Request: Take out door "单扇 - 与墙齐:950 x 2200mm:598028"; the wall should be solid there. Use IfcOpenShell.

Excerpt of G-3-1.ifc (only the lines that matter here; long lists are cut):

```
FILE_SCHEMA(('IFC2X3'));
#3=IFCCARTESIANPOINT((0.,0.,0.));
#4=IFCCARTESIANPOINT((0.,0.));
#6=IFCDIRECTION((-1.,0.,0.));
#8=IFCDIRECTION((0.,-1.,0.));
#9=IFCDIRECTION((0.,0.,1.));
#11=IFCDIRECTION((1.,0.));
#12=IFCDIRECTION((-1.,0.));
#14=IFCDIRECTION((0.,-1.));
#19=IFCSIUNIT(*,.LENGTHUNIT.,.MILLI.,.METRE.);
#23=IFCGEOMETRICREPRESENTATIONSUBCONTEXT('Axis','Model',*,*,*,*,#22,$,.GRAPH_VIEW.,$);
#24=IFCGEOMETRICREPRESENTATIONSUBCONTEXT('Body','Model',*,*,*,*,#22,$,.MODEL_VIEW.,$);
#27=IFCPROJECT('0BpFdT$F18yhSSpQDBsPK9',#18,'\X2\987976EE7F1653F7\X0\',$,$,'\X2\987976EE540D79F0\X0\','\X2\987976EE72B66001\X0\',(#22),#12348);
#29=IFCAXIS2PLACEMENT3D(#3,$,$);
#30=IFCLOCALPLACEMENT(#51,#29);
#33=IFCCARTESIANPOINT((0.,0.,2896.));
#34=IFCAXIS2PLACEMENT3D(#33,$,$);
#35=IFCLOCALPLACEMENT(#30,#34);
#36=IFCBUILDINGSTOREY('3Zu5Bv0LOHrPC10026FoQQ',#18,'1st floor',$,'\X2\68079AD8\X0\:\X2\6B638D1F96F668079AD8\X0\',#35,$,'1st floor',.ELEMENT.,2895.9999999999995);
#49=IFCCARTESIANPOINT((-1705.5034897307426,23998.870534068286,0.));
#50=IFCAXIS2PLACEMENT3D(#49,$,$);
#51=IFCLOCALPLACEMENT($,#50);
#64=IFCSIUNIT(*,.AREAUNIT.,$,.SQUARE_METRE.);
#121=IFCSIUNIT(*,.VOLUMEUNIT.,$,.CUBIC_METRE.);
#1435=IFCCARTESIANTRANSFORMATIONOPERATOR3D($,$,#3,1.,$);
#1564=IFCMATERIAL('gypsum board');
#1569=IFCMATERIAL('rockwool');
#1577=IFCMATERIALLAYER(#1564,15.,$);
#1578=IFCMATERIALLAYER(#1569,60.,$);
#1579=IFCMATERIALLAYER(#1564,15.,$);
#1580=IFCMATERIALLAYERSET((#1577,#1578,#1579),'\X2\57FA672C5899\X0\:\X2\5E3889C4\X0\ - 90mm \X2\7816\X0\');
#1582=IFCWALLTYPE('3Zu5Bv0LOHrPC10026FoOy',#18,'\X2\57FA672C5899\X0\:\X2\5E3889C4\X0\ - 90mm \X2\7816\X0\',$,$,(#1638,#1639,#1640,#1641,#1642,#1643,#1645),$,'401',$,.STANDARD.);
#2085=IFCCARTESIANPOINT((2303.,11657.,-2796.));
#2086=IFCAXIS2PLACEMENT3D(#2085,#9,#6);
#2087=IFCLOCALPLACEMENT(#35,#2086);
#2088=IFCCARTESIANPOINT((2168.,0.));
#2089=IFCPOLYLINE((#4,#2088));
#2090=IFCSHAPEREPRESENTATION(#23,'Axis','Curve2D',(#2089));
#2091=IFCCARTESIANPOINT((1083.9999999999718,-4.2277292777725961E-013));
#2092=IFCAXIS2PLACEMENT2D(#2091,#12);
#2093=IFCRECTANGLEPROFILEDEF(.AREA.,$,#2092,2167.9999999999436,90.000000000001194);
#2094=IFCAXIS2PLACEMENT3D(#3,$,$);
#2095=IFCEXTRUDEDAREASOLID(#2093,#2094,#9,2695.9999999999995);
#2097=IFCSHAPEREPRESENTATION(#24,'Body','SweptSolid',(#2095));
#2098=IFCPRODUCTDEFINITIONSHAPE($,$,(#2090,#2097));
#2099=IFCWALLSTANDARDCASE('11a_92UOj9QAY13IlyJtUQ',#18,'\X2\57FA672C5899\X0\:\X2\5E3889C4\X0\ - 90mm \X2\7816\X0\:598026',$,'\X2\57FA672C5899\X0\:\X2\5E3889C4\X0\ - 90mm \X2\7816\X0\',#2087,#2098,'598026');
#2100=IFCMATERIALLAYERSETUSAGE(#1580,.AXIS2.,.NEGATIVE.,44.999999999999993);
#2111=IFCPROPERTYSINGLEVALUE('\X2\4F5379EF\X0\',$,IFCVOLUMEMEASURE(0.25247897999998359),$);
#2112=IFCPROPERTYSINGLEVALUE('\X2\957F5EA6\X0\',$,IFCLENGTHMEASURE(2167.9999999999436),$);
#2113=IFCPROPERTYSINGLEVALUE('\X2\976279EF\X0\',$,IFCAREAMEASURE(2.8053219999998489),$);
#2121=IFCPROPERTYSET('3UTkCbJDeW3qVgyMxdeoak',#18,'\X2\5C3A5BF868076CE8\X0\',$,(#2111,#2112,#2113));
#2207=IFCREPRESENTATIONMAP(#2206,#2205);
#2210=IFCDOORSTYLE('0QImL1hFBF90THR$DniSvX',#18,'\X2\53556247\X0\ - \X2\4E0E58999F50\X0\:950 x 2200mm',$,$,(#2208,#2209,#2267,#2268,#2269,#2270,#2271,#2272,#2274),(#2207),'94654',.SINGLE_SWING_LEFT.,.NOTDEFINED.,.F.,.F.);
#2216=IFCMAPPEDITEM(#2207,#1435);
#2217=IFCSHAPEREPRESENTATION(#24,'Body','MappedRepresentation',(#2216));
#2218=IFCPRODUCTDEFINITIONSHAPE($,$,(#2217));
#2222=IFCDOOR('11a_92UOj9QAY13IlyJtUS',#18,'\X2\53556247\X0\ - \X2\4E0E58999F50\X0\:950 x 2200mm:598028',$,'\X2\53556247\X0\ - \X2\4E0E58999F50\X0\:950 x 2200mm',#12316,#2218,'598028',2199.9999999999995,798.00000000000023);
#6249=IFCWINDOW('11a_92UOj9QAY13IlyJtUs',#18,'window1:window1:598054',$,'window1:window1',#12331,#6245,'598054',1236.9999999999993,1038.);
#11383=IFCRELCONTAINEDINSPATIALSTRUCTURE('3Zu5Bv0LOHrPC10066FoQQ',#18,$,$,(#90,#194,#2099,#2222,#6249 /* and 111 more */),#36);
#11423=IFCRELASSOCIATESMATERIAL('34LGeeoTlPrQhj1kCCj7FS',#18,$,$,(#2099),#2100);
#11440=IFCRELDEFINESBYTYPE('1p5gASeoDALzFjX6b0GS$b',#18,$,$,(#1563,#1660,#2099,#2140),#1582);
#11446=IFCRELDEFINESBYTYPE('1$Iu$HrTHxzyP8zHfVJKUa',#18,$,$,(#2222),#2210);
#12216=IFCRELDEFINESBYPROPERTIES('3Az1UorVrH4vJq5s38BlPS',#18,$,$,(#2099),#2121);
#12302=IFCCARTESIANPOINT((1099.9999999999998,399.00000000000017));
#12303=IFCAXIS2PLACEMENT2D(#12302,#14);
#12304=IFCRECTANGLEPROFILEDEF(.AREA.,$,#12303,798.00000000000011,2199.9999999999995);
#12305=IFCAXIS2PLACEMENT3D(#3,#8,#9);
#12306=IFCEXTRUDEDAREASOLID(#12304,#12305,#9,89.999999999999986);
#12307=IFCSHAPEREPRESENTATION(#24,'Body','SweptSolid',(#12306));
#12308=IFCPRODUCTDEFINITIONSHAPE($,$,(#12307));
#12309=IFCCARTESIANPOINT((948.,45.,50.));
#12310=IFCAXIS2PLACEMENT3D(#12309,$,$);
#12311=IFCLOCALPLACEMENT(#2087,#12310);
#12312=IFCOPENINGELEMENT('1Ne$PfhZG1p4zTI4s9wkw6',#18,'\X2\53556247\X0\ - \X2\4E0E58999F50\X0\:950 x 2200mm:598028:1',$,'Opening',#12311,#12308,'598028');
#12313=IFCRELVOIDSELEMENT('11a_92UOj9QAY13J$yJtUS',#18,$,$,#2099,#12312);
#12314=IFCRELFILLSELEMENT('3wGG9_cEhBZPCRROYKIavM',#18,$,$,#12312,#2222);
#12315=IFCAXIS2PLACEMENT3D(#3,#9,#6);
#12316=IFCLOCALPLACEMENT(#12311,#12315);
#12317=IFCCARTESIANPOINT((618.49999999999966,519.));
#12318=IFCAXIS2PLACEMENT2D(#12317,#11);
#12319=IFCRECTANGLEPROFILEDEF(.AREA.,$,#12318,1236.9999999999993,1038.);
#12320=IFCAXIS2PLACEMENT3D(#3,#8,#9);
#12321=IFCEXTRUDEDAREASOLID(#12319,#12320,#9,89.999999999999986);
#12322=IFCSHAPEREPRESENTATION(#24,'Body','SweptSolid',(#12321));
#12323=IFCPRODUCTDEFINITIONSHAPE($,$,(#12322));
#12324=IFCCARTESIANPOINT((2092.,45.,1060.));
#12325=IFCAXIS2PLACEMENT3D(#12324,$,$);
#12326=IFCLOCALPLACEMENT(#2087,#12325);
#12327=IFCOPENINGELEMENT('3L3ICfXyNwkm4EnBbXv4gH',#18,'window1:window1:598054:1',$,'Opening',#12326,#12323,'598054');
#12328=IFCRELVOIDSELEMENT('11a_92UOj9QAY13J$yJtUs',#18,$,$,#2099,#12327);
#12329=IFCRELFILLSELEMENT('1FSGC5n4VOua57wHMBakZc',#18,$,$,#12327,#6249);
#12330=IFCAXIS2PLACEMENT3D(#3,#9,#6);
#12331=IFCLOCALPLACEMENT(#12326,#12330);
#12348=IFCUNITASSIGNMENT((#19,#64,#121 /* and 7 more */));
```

```python
import ifcopenshell
import ifcopenshell.api.feature
import ifcopenshell.api.pset
import ifcopenshell.api.root
import ifcopenshell.geom
import ifcopenshell.util.element
import ifcopenshell.util.shape
import ifcopenshell.util.unit

model = ifcopenshell.open("G-3-1.ifc")
area_scale = ifcopenshell.util.unit.calculate_unit_scale(model, "AREAUNIT")
volume_scale = ifcopenshell.util.unit.calculate_unit_scale(model, "VOLUMEUNIT")
settings = ifcopenshell.geom.settings()


def volume(element):
    """Net volume in cubic metres, openings subtracted."""
    shape = ifcopenshell.geom.create_shape(settings, element)
    return ifcopenshell.util.shape.get_volume(shape.geometry)


door = model.by_id(2222)
opening = door.FillsVoids[0].RelatingOpeningElement
wall = opening.VoidsElements[0].RelatingBuildingElement
before = volume(wall)

ifcopenshell.api.root.remove_product(model, product=door)
ifcopenshell.api.feature.remove_feature(model, feature=opening)

after = volume(wall)
thickness = 0.09  # wall thickness in metres

# Update the wall's stored quantities.
pset = model.by_id(ifcopenshell.util.element.get_pset(wall, "尺寸标注", should_inherit=False)["id"])
ifcopenshell.api.pset.edit_pset(model, pset=pset, properties={
    "体积": model.create_entity("IfcVolumeMeasure", after / volume_scale),
    "面积": model.create_entity("IfcAreaMeasure", after / thickness / area_scale),
})

print(f"wall volume {before:.3f} -> {after:.3f} m3")

model.write("G-3-1_v2.ifc")
```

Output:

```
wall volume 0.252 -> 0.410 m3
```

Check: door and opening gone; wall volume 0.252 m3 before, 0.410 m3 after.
